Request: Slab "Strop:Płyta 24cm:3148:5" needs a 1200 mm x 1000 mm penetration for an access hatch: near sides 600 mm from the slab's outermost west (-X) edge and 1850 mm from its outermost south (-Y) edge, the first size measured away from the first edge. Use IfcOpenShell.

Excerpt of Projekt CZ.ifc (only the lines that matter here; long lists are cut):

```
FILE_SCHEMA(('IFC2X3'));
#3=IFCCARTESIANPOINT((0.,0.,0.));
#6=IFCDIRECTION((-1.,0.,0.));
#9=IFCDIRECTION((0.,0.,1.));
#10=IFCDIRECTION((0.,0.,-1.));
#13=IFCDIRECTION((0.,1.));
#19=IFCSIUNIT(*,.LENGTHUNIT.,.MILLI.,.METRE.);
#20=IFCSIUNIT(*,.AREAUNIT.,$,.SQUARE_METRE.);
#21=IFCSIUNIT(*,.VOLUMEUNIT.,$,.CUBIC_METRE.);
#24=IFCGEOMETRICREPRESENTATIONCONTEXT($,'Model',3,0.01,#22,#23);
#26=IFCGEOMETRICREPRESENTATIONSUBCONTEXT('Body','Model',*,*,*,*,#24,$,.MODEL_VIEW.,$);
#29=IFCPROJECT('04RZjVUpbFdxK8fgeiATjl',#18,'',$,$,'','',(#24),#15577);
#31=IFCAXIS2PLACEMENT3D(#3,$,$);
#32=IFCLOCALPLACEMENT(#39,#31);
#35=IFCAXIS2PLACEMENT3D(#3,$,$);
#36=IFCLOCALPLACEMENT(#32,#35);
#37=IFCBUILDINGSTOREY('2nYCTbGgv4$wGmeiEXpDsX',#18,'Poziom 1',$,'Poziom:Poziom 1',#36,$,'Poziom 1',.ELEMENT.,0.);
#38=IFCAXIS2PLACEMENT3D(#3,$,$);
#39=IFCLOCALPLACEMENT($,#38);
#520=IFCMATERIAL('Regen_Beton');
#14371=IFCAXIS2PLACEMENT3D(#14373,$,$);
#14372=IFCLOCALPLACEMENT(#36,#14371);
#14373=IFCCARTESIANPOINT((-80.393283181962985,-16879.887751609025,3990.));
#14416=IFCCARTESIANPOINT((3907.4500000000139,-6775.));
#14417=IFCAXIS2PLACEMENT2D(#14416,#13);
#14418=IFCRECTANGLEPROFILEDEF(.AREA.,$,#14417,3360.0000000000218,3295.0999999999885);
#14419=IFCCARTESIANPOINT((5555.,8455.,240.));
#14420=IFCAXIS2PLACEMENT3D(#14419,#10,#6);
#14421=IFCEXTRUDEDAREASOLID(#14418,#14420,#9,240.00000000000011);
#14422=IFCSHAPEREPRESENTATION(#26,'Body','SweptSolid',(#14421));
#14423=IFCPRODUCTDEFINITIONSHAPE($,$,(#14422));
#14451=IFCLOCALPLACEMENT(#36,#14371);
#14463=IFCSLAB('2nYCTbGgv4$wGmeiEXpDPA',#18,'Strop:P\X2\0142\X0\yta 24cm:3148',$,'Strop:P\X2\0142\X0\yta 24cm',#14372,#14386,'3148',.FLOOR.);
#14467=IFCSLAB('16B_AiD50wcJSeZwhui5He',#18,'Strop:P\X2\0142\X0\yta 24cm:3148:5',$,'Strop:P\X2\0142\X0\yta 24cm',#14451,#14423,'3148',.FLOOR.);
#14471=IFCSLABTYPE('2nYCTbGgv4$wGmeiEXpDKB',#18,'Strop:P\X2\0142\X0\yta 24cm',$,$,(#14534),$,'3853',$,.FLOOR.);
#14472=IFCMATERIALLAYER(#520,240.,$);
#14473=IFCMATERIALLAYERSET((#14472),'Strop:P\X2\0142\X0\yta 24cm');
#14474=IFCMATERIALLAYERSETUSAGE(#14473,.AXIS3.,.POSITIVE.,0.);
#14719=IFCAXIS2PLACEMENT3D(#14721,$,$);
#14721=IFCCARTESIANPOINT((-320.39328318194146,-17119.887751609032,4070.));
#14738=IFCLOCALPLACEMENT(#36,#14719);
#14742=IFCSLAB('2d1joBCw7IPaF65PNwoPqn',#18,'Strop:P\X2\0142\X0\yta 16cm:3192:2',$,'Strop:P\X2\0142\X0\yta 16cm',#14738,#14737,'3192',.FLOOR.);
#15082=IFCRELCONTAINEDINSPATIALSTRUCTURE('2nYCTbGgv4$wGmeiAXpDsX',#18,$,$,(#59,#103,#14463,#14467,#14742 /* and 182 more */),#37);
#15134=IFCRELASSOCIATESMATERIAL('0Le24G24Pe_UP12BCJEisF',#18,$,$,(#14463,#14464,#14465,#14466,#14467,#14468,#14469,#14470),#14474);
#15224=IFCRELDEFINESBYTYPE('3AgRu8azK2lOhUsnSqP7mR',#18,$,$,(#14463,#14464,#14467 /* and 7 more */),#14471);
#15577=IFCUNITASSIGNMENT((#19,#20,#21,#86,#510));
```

```python
import numpy as np
import ifcopenshell
import ifcopenshell.api.feature
import ifcopenshell.api.geometry
import ifcopenshell.api.root
import ifcopenshell.geom
import ifcopenshell.util.placement
import ifcopenshell.util.representation
import ifcopenshell.util.shape
import ifcopenshell.util.unit

model = ifcopenshell.open("Projekt CZ.ifc")
unit_scale = ifcopenshell.util.unit.calculate_unit_scale(model)
settings = ifcopenshell.geom.settings()


def volume(element):
    """Net volume in cubic metres, openings subtracted."""
    shape = ifcopenshell.geom.create_shape(settings, element)
    return ifcopenshell.util.shape.get_volume(shape.geometry)


slab = model.by_guid("16B_AiD50wcJSeZwhui5He")
before = volume(slab)

# Extent in the slab's own axes, in metres. The edges named are its -X and -Y sides.
slab_shape = ifcopenshell.geom.create_shape(settings, slab)
vertices = ifcopenshell.util.shape.get_vertices(slab_shape.geometry)
x_min, y_min, bottom = vertices.min(axis=0)
top = vertices[:, 2].max()

opening = ifcopenshell.api.root.create_entity(model, ifc_class="IfcOpeningElement", name="Access hatch opening")
context = ifcopenshell.util.representation.get_context(model, "Model", "Body", "MODEL_VIEW")
width, depth = 1.2, 1
outline = [(0.0, 0.0), (width, 0.0), (width, depth), (0.0, depth), (0.0, 0.0)]
# Overshoot both faces by 50 mm so the cut is clean.
shape = ifcopenshell.api.geometry.add_slab_representation(
    model, context=context, depth=top - bottom + 0.1, polyline=outline
)
ifcopenshell.api.geometry.assign_representation(model, product=opening, representation=shape)

matrix = ifcopenshell.util.placement.get_local_placement(slab.ObjectPlacement)
matrix[:, 3] = matrix @ np.append(np.array([x_min + 0.6, y_min + 1.85, bottom - 0.05]) / unit_scale, 1.0)
ifcopenshell.api.geometry.edit_object_placement(model, product=opening, matrix=matrix, is_si=False)
ifcopenshell.api.feature.add_feature(model, feature=opening, element=slab)

after = volume(slab)

print(f"slab volume {before:.3f} -> {after:.3f} m3")

model.write("Projekt CZ_updated.ifc")
```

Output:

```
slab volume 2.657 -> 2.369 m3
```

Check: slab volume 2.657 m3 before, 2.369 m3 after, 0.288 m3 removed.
